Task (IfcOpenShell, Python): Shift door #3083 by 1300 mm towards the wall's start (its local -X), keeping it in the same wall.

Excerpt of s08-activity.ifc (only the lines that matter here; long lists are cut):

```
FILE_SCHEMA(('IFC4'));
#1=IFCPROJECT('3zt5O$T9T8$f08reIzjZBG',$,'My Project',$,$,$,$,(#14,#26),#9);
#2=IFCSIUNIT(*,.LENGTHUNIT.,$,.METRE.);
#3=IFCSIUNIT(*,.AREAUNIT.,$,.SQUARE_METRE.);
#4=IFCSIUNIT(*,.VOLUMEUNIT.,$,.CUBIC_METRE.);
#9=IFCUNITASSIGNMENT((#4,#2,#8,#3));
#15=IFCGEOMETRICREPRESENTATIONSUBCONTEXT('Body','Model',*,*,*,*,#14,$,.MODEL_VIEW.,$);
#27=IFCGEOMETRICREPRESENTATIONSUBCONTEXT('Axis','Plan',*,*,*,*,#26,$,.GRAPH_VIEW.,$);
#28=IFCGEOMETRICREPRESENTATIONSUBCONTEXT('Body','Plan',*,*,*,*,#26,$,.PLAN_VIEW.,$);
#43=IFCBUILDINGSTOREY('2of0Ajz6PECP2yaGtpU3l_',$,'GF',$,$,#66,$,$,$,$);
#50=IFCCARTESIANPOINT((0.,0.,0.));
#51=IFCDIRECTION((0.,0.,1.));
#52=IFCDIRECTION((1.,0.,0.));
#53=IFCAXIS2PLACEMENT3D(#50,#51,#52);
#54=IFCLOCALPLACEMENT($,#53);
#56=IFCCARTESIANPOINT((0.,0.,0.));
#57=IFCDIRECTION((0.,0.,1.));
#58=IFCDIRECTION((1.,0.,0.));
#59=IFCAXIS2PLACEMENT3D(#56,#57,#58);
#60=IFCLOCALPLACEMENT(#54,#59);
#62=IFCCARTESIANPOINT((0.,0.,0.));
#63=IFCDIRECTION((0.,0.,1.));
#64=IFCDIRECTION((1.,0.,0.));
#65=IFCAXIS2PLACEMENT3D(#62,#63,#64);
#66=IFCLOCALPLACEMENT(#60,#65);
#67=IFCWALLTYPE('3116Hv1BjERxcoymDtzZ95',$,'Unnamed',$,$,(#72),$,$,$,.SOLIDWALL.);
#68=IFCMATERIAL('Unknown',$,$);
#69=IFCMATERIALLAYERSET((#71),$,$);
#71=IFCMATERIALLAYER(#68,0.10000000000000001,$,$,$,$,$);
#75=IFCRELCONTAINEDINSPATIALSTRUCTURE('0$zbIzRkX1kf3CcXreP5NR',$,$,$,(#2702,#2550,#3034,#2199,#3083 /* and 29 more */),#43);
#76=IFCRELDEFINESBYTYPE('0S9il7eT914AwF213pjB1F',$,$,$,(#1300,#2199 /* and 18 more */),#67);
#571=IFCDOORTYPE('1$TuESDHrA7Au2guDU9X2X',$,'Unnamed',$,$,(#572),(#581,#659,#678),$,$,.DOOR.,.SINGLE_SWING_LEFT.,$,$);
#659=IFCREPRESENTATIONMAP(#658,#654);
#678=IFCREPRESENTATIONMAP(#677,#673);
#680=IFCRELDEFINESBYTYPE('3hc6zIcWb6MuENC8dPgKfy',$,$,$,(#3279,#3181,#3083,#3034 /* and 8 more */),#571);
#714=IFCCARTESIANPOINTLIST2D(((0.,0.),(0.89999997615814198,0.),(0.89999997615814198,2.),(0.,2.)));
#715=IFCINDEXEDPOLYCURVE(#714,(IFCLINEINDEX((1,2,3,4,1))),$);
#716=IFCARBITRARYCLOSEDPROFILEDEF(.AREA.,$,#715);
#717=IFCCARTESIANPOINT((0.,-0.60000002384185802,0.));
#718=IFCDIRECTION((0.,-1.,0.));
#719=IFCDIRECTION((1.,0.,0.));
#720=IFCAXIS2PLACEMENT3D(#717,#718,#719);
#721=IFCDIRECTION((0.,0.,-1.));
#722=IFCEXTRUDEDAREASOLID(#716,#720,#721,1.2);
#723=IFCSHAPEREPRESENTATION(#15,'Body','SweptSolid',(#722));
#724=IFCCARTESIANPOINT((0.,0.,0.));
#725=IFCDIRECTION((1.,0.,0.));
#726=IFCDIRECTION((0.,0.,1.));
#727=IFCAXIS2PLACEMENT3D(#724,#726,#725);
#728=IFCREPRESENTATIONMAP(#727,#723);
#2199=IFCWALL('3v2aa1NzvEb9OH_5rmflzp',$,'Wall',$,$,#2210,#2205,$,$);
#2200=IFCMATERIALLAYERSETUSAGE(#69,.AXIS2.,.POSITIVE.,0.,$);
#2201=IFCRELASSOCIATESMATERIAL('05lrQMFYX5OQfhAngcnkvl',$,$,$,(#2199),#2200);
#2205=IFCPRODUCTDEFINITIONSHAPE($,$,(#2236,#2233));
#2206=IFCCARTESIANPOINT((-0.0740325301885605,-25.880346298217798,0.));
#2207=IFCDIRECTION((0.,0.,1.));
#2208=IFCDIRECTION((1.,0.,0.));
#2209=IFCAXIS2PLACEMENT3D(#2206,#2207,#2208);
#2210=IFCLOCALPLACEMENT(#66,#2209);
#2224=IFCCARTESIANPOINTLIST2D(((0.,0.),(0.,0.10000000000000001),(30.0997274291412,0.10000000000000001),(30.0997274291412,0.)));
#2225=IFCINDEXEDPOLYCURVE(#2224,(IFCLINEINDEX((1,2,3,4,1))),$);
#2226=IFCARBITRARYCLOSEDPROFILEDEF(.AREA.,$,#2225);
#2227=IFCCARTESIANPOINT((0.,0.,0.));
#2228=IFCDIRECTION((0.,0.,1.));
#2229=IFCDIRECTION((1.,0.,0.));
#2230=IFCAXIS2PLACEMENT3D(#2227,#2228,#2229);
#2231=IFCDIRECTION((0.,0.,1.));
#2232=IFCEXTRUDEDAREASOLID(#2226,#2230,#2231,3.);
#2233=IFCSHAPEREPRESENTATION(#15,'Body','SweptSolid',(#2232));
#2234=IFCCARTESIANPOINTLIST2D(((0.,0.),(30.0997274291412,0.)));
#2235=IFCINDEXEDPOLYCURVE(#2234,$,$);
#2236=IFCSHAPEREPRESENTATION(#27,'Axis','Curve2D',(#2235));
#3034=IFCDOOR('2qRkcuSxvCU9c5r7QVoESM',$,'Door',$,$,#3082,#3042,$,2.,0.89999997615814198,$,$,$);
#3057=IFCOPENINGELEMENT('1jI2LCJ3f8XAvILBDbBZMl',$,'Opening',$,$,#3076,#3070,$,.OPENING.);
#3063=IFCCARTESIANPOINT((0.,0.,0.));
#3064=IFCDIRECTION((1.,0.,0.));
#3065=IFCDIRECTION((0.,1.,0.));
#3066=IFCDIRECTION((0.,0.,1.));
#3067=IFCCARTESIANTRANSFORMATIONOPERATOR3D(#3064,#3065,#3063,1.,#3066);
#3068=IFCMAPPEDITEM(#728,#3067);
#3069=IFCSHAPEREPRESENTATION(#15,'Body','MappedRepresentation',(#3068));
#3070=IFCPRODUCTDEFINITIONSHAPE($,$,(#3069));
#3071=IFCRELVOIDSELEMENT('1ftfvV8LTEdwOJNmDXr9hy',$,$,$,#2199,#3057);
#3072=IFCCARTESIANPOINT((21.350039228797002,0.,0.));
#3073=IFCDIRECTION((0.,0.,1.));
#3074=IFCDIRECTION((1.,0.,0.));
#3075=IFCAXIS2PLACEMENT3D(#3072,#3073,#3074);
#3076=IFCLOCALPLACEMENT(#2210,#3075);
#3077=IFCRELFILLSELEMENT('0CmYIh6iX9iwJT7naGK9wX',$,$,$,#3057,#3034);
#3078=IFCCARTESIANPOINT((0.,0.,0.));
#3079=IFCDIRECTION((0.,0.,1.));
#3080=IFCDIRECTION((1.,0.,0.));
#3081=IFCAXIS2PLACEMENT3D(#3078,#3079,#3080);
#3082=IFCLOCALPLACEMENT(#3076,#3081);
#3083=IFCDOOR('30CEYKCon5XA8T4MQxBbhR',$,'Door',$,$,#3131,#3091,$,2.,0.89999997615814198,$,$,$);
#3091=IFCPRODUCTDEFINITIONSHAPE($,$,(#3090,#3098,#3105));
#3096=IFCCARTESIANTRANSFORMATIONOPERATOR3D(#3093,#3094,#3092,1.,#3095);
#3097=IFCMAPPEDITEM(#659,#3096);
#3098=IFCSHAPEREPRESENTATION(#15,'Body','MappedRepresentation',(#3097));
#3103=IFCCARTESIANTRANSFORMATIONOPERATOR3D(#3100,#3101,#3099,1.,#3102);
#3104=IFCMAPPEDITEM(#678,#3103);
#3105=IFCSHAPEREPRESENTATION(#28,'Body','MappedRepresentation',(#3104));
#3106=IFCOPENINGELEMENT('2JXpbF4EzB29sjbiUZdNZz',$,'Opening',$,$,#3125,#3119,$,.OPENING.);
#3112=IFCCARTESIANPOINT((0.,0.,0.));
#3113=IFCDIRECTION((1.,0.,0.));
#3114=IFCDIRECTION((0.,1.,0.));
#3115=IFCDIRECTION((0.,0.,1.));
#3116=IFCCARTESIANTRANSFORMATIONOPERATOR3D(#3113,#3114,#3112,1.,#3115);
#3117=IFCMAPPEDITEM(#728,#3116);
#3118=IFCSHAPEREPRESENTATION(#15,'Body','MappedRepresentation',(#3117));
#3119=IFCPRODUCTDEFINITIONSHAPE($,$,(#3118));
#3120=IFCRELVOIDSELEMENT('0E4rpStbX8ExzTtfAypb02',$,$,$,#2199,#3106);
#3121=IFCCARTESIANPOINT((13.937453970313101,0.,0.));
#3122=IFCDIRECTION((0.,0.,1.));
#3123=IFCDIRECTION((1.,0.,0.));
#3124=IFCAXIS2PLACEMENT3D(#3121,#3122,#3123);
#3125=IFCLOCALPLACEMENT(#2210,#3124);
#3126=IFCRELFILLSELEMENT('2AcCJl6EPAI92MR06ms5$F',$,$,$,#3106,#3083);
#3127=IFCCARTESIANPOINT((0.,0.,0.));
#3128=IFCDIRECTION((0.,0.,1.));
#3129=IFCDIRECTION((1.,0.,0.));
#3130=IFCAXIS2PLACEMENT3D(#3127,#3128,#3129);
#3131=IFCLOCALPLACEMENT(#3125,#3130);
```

```python
import ifcopenshell
import ifcopenshell.api.geometry
import ifcopenshell.util.placement
import ifcopenshell.util.unit

model = ifcopenshell.open("s08-activity.ifc")
unit_scale = ifcopenshell.util.unit.calculate_unit_scale(model)

door = model.by_guid("30CEYKCon5XA8T4MQxBbhR")
opening = door.FillsVoids[0].RelatingOpeningElement
wall = opening.VoidsElements[0].RelatingBuildingElement

wall_matrix = ifcopenshell.util.placement.get_local_placement(wall.ObjectPlacement)
shift = wall_matrix[:3, 0] * -1.3 / unit_scale
before = ifcopenshell.util.placement.get_local_placement(door.ObjectPlacement)[:3, 3].copy()

# The door is placed relative to its opening, so it follows when the opening moves.
matrix = ifcopenshell.util.placement.get_local_placement(opening.ObjectPlacement)
matrix[:3, 3] += shift
ifcopenshell.api.geometry.edit_object_placement(
    model, product=opening, matrix=matrix, is_si=False, should_transform_children=True
)

after = ifcopenshell.util.placement.get_local_placement(door.ObjectPlacement)[:3, 3]
print("door moved by", (after - before).round(3) + 0.0)

model.write("s08-activity_rev.ifc")
```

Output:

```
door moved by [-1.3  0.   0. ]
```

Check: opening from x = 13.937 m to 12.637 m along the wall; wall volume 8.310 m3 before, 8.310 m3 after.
